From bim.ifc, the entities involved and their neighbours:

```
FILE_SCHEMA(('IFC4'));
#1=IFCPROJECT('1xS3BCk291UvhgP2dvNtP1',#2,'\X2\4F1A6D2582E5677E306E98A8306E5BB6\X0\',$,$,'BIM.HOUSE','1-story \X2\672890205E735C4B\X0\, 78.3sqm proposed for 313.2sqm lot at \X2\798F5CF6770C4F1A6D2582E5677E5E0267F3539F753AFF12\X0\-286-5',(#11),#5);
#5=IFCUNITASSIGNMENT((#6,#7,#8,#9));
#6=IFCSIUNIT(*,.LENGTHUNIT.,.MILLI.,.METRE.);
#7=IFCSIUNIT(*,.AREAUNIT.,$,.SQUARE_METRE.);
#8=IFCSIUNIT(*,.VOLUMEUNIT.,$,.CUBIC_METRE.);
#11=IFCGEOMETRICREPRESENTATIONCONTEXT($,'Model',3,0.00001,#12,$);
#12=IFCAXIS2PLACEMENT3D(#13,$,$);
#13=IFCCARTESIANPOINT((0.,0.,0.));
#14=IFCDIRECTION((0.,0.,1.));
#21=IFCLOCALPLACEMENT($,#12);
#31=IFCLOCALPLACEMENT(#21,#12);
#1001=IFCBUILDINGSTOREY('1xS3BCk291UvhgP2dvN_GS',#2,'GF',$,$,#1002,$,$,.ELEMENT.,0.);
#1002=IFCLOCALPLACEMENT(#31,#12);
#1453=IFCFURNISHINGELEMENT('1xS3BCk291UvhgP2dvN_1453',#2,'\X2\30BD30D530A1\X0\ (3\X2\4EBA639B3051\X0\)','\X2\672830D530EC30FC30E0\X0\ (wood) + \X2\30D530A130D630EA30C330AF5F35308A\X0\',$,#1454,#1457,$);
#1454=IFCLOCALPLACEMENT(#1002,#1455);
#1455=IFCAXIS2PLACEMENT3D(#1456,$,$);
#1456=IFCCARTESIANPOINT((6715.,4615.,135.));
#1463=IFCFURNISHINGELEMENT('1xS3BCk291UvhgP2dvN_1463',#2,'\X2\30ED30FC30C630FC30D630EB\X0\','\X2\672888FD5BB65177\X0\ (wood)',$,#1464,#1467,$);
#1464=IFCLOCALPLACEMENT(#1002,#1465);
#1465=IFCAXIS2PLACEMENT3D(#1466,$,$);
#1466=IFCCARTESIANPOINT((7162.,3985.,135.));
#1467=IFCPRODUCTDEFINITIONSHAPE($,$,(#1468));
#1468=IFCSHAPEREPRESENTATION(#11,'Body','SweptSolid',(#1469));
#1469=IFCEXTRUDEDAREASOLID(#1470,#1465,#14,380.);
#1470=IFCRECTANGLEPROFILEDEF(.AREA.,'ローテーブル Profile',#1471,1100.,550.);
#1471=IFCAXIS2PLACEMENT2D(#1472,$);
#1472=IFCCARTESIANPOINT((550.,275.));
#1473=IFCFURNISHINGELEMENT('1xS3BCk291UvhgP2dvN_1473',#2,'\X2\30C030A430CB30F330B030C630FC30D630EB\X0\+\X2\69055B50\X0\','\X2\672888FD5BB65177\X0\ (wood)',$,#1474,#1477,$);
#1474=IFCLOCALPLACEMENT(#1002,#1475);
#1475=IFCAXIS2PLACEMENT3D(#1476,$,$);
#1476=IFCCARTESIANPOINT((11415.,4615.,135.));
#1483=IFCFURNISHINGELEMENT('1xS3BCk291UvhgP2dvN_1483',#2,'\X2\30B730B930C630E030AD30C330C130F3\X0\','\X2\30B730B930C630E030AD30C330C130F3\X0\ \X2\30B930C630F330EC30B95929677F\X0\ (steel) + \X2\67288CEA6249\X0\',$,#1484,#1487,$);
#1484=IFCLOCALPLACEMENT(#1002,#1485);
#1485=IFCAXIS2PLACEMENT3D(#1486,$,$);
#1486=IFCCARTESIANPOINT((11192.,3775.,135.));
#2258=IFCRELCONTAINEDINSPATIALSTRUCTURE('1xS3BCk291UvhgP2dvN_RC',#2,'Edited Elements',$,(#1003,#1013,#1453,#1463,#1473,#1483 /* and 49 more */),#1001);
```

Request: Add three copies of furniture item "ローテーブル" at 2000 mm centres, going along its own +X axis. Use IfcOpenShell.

```python
import ifcopenshell
import ifcopenshell.api.geometry
import ifcopenshell.api.root
import ifcopenshell.util.element
import ifcopenshell.util.placement

model = ifcopenshell.open("bim.ifc")


def reuse_history(source, copy):
    """copy_class also copies each property set's owner history, people and application; keep the originals."""
    for rel in copy.IsDefinedBy:
        if rel.is_a("IfcRelDefinesByProperties") and (history := rel.RelatingPropertyDefinition.OwnerHistory):
            rel.RelatingPropertyDefinition.OwnerHistory = source.OwnerHistory
            ifcopenshell.util.element.remove_deep2(model, history)


source = model.by_guid("1xS3BCk291UvhgP2dvN_1463")
base = ifcopenshell.util.placement.get_local_placement(source.ObjectPlacement)
step = base[:3, 0] * 2000.0

for i in range(1, 4):
    copy = ifcopenshell.api.root.copy_class(model, product=source)
    copy.Representation = ifcopenshell.util.element.copy_deep(
        model, source.Representation, exclude=["IfcGeometricRepresentationContext", "IfcRepresentationMap"]
    )
    reuse_history(source, copy)
    matrix = base.copy()
    matrix[:3, 3] += i * step
    print("added at", matrix[:3, 3].round(3) + 0.0)
    ifcopenshell.api.geometry.edit_object_placement(model, product=copy, matrix=matrix, is_si=False)

model.write("bim_v2.ifc")
```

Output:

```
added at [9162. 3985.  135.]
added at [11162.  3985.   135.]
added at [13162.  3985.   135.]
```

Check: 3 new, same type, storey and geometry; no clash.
